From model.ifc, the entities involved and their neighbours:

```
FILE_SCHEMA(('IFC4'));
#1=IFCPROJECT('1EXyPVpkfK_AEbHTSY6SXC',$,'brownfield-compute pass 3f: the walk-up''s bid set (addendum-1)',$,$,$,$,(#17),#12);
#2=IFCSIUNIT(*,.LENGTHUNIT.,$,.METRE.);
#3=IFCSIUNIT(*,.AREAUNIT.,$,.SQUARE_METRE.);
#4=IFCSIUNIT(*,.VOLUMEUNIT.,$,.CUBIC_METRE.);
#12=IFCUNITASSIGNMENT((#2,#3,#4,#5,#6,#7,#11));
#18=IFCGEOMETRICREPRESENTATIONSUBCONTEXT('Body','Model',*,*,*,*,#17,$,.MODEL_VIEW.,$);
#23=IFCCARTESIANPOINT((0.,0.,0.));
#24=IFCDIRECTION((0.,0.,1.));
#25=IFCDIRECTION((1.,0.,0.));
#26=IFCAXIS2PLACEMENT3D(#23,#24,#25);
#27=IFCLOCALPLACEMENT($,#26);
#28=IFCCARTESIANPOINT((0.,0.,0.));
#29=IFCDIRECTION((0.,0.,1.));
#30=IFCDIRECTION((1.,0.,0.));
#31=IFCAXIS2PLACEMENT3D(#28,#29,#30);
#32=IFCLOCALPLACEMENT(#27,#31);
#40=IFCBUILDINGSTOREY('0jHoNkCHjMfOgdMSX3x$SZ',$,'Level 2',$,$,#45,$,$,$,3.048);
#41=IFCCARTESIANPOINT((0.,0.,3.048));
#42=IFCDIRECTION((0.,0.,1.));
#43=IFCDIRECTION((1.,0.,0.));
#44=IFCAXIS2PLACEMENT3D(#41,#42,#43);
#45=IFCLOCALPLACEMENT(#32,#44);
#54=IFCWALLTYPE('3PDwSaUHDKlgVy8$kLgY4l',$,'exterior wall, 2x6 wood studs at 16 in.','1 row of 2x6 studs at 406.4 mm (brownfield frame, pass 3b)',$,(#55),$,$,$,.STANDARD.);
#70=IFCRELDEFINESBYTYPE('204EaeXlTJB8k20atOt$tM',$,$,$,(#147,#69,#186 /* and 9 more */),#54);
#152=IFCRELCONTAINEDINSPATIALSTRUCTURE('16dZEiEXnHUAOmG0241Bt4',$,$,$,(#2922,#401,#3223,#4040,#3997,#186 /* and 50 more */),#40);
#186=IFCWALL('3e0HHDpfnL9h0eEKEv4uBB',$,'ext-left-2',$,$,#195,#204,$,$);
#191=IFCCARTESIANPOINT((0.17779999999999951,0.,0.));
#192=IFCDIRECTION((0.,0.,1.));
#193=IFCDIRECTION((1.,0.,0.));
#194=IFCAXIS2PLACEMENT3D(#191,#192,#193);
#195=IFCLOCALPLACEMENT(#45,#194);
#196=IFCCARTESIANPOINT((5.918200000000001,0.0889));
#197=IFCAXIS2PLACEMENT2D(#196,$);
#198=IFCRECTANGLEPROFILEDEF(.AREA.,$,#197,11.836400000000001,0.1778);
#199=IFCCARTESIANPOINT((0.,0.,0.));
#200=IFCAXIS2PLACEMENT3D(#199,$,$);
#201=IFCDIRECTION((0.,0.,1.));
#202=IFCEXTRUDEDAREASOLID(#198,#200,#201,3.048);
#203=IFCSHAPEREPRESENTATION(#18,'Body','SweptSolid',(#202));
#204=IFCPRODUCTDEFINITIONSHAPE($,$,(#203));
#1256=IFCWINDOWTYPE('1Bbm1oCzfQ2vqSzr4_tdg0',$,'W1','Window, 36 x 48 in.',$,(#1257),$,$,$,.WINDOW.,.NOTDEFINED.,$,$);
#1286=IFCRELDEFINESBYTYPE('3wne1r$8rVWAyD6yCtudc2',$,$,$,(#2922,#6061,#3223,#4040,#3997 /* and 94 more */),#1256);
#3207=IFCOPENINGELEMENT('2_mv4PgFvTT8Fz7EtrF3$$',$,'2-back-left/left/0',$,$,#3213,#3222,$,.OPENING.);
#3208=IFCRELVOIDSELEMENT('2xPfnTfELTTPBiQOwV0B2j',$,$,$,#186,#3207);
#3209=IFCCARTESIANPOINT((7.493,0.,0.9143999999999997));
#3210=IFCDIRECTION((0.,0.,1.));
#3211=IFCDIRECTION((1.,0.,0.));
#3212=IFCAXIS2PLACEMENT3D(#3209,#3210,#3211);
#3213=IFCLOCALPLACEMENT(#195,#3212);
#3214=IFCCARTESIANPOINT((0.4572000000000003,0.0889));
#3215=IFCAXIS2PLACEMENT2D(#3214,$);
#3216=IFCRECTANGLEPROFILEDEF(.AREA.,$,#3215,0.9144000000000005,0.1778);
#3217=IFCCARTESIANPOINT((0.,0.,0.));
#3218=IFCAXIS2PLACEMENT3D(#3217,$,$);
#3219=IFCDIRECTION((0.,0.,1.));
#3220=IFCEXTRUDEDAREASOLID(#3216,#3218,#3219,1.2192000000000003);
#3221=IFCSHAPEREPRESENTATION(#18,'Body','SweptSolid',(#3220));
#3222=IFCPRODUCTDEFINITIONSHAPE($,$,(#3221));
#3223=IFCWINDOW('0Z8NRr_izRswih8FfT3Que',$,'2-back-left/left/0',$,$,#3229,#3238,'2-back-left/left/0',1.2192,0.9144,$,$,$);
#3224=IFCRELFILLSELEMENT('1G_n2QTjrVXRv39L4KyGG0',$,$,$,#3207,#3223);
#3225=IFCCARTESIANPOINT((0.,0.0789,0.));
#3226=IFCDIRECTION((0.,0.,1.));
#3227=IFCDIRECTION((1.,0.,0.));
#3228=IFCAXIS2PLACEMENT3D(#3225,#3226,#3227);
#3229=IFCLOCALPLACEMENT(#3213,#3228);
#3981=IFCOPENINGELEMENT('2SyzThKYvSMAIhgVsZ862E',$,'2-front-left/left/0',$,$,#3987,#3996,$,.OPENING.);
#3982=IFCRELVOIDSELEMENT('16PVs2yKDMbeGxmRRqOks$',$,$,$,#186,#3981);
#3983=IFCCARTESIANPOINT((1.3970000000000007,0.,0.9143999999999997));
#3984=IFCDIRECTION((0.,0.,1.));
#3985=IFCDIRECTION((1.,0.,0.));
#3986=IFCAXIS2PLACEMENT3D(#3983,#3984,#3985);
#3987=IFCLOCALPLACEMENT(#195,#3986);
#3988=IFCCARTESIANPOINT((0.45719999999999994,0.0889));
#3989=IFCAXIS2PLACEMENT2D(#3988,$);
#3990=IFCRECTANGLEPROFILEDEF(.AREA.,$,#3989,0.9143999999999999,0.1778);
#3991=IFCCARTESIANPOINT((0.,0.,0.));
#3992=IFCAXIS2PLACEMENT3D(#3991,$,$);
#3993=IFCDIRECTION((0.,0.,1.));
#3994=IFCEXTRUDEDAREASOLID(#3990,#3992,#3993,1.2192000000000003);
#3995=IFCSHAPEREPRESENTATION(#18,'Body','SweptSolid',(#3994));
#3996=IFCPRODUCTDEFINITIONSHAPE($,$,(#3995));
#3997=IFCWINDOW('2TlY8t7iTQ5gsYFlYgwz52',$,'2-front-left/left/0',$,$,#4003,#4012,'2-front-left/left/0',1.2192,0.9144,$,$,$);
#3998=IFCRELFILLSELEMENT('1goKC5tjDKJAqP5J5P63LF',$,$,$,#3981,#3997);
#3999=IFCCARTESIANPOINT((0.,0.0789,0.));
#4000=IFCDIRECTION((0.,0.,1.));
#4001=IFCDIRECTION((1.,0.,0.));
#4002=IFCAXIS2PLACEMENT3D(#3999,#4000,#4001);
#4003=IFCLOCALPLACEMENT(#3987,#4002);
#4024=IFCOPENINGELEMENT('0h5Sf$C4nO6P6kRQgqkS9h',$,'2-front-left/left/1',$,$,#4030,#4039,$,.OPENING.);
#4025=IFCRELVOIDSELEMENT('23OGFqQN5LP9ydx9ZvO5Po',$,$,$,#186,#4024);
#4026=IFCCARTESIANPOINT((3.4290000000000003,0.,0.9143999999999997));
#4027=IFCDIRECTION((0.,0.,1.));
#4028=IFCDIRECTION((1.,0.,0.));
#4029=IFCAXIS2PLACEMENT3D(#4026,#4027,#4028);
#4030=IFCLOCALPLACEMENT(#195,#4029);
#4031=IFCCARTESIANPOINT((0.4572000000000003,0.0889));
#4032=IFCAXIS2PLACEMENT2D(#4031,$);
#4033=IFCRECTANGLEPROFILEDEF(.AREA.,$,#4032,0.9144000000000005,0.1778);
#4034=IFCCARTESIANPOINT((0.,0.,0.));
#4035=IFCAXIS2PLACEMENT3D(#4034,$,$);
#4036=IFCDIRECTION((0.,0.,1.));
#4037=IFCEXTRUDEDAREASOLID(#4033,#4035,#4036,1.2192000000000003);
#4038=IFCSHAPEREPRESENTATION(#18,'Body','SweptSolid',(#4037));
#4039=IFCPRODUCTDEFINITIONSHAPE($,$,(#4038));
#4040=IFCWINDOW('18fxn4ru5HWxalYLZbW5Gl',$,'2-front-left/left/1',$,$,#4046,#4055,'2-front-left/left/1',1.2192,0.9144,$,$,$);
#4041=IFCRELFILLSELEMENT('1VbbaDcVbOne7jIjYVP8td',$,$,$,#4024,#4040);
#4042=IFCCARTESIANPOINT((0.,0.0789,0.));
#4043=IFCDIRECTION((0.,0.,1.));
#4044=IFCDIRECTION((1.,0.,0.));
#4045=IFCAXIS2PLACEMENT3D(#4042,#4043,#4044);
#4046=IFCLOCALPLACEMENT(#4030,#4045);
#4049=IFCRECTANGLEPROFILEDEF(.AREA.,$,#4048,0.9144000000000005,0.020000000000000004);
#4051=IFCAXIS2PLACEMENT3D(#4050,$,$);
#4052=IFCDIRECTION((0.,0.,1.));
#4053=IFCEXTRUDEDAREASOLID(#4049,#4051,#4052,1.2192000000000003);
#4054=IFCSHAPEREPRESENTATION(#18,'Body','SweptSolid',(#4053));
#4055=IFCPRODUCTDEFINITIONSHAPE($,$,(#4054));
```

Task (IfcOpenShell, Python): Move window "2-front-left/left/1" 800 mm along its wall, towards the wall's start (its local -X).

```python
import ifcopenshell
import ifcopenshell.api.geometry
import ifcopenshell.util.placement

model = ifcopenshell.open("model.ifc")

window = model.by_guid("18fxn4ru5HWxalYLZbW5Gl")
opening = window.FillsVoids[0].RelatingOpeningElement
wall = opening.VoidsElements[0].RelatingBuildingElement

wall_matrix = ifcopenshell.util.placement.get_local_placement(wall.ObjectPlacement)
shift = wall_matrix[:3, 0] * -0.8
before = ifcopenshell.util.placement.get_local_placement(window.ObjectPlacement)[:3, 3].copy()

# The window is placed relative to its opening, so it follows when the opening moves.
matrix = ifcopenshell.util.placement.get_local_placement(opening.ObjectPlacement)
matrix[:3, 3] += shift
ifcopenshell.api.geometry.edit_object_placement(
    model, product=opening, matrix=matrix, is_si=False, should_transform_children=True
)

after = ifcopenshell.util.placement.get_local_placement(window.ObjectPlacement)[:3, 3]
print("window moved by", (after - before).round(3) + 0.0)

model.write("model_v2.ifc")
```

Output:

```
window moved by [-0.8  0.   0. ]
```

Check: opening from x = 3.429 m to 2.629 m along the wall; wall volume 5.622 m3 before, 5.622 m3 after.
